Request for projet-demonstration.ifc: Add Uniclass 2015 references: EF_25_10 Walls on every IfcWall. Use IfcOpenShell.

First a look at what the model holds.

```python
import ifcopenshell

model = ifcopenshell.open("projet-demonstration.ifc")
print(model.schema)
print("classifications:", [c.Name for c in model.by_type("IfcClassification")])
for ifc_class in ("IfcDoor", "IfcRoof", "IfcStair", "IfcWall", "IfcWindow"):
    print(ifc_class, len(model.by_type(ifc_class)))
```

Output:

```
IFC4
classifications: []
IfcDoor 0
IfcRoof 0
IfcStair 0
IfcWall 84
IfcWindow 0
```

```python
import ifcopenshell
import ifcopenshell.api.classification

model = ifcopenshell.open("projet-demonstration.ifc")

system = ifcopenshell.api.classification.add_classification(model, classification="Uniclass 2015")

codes = {
    "IfcWall": ("EF_25_10", "Walls"),
}
for ifc_class, (code, name) in codes.items():
    products = model.by_type(ifc_class)
    ifcopenshell.api.classification.add_reference(
        model, products=products, classification=system, identification=code, name=name
    )
    print(code, len(products))

model.write("projet-demonstration_edited.ifc")
```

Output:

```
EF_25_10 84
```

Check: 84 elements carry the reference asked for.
